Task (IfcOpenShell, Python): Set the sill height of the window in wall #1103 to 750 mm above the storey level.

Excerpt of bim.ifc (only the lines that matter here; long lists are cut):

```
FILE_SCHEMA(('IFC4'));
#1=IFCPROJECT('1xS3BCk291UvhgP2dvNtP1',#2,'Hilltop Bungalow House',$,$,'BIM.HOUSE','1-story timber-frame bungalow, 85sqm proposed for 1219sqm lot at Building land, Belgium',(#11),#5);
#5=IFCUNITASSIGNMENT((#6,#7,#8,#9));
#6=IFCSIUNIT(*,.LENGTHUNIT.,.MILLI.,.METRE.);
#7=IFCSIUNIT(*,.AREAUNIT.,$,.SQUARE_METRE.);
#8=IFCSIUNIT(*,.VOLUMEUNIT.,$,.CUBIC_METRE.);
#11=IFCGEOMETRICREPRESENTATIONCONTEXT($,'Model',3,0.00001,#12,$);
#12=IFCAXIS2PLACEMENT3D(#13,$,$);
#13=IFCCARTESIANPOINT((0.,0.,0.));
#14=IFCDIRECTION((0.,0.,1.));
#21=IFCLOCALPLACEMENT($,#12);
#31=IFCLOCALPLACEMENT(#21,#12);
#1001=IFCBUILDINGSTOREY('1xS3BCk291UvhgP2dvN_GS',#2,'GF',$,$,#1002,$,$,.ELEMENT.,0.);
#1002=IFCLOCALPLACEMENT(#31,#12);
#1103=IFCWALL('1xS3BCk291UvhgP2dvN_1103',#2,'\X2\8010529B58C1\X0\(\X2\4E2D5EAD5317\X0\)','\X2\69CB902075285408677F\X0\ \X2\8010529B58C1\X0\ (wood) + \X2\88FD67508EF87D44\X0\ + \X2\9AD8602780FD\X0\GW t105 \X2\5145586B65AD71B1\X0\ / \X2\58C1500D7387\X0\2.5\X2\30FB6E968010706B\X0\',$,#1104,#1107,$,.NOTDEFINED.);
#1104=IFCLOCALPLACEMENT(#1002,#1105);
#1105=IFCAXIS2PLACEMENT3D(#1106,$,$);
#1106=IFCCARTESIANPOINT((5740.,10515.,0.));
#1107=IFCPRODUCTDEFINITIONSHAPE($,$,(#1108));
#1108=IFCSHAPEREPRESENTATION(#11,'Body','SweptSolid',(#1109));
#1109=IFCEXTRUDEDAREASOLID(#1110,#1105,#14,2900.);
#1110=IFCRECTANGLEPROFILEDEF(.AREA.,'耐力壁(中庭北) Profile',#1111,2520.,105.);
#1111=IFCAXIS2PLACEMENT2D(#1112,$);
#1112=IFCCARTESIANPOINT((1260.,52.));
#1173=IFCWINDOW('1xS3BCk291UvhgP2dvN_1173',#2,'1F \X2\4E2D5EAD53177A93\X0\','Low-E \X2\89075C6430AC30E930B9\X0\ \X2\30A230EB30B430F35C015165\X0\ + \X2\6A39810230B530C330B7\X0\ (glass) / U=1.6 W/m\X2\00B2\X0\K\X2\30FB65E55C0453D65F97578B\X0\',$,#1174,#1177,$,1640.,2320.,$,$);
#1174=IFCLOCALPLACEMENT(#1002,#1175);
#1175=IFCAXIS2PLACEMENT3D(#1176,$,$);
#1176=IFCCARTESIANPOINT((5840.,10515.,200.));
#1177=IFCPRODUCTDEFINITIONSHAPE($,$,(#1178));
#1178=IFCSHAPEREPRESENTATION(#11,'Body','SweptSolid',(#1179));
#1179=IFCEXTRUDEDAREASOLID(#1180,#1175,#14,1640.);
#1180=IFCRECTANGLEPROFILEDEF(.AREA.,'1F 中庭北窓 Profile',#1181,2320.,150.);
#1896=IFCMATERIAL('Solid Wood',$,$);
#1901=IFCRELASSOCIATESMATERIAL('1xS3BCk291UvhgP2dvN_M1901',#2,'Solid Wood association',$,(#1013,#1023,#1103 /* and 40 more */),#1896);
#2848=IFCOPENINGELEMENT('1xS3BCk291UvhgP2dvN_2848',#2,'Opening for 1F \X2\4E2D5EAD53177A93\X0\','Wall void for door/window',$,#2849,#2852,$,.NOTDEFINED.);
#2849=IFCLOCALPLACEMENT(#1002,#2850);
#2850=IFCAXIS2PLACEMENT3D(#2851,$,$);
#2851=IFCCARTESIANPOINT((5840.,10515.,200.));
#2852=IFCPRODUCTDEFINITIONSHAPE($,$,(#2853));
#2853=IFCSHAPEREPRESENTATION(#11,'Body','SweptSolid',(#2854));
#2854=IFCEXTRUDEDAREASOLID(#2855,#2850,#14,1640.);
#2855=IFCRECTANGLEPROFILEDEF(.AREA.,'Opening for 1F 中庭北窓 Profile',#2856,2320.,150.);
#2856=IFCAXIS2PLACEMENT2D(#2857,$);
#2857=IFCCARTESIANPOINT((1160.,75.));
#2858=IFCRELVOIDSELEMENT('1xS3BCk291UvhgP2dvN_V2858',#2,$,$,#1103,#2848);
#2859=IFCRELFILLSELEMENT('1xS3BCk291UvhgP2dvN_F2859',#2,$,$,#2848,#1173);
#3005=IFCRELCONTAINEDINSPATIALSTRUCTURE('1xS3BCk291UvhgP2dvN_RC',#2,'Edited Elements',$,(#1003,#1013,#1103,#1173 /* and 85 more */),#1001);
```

```python
import numpy as np
import ifcopenshell
import ifcopenshell.api.geometry
import ifcopenshell.geom
import ifcopenshell.util.element
import ifcopenshell.util.placement
import ifcopenshell.util.shape
import ifcopenshell.util.unit

model = ifcopenshell.open("bim.ifc")
unit_scale = ifcopenshell.util.unit.calculate_unit_scale(model)

window = model.by_guid("1xS3BCk291UvhgP2dvN_1173")
opening = window.FillsVoids[0].RelatingOpeningElement
storey = ifcopenshell.util.element.get_container(window, ifc_class="IfcBuildingStorey")
level = ifcopenshell.util.placement.get_local_placement(storey.ObjectPlacement)[2, 3]

# The opening's origin need not be at the sill, so measure its lowest point.
shape = ifcopenshell.geom.create_shape(ifcopenshell.geom.settings(), opening)
bottom = ifcopenshell.util.shape.get_shape_bottom_elevation(shape, shape.geometry) / unit_scale
dz = level + 750.0 - bottom

shift = np.array([0.0, 0.0, dz])
# The window is not placed relative to its opening, so move both.
for product in (opening, window):
    matrix = ifcopenshell.util.placement.get_local_placement(product.ObjectPlacement)
    matrix[:3, 3] += shift
    ifcopenshell.api.geometry.edit_object_placement(model, product=product, matrix=matrix, is_si=False)

print(f"moved by {dz * unit_scale:+.3f} m")

model.write("bim-out.ifc")
```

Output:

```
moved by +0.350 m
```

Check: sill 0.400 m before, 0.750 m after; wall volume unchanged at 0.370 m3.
